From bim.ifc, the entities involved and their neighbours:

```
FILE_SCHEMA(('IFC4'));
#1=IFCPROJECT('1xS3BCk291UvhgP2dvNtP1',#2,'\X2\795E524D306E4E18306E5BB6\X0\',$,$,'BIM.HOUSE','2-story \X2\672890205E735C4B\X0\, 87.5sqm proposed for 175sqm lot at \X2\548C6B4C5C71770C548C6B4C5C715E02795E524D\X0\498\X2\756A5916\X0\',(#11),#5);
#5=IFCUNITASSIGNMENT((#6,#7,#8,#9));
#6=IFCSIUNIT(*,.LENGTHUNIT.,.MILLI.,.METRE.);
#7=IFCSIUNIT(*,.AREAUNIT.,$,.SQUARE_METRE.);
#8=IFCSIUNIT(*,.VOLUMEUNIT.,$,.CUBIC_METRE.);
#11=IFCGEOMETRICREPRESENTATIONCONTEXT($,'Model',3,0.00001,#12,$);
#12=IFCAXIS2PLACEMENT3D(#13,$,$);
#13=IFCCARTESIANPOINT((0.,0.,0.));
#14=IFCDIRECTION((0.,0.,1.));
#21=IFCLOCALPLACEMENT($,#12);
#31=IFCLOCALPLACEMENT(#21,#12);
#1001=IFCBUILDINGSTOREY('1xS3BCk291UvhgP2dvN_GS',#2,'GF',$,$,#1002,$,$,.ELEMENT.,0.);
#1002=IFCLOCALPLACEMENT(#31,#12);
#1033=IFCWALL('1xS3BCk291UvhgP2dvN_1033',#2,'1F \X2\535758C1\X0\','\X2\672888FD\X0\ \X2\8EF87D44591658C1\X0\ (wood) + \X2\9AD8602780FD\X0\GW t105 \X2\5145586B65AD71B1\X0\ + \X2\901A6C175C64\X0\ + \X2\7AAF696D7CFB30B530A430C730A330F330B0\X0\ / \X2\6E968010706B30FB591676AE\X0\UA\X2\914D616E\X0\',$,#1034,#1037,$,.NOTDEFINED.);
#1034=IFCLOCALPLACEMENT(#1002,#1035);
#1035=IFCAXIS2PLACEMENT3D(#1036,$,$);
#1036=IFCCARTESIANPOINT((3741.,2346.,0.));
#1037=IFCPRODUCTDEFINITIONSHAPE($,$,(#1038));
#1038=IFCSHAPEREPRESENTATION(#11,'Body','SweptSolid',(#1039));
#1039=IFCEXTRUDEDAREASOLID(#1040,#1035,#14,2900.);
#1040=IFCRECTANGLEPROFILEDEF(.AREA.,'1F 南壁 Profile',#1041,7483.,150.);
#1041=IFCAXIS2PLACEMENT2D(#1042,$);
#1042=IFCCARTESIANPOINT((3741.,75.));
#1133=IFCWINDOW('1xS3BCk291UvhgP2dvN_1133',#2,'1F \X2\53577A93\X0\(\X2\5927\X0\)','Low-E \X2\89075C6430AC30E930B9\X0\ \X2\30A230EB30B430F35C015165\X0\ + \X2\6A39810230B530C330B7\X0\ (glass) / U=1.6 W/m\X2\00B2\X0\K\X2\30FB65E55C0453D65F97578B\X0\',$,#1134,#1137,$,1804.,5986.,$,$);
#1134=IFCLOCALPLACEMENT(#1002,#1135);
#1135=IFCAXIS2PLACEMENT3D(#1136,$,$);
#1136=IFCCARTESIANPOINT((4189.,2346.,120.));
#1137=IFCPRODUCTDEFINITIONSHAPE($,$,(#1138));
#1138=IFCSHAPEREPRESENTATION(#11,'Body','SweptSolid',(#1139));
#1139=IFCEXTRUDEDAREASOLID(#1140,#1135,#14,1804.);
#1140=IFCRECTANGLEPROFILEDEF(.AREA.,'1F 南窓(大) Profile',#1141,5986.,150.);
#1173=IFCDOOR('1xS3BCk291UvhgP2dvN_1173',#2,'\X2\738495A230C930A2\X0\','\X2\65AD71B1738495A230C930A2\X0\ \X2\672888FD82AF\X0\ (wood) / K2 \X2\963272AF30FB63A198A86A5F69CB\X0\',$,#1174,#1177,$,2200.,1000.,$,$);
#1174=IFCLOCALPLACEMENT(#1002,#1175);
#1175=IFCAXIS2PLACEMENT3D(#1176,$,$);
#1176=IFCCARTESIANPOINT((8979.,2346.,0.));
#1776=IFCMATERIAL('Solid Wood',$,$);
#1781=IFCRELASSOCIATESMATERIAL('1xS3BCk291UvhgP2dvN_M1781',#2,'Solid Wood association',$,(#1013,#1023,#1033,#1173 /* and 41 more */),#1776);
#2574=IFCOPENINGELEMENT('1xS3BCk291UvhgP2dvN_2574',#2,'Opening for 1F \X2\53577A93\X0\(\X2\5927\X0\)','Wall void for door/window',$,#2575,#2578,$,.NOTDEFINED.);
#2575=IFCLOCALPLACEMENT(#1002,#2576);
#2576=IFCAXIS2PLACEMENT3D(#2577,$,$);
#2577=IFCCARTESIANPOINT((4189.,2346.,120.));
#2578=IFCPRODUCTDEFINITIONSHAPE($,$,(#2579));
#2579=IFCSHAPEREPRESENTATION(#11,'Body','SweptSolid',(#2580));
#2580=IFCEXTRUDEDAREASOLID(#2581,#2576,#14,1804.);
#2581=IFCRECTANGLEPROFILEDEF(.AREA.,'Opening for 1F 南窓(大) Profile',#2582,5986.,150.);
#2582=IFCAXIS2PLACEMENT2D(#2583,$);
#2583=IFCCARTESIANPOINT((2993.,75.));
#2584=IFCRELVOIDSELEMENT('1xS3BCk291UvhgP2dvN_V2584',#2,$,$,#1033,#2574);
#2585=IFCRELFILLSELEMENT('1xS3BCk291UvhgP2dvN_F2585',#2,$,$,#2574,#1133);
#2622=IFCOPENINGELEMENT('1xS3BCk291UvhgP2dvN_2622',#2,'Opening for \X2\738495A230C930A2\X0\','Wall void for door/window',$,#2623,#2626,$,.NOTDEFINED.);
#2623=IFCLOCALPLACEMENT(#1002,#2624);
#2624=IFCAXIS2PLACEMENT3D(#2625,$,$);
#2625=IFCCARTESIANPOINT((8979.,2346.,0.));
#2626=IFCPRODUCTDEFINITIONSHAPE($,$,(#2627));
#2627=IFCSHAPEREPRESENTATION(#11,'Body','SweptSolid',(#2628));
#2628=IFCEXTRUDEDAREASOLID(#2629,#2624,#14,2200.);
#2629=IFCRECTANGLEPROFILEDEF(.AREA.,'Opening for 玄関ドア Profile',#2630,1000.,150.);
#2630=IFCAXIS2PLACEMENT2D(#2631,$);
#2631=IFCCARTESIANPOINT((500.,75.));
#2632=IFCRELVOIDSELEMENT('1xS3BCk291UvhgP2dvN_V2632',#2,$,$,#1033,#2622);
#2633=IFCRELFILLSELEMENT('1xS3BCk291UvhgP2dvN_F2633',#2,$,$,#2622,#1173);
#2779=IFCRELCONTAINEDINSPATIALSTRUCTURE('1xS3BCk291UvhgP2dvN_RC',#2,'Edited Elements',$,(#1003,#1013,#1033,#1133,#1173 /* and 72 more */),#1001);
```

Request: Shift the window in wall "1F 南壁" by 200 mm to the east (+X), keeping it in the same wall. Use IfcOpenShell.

```python
import ifcopenshell
import ifcopenshell.api.geometry
import ifcopenshell.util.placement
import ifcopenshell.util.unit

model = ifcopenshell.open("bim.ifc")
unit_scale = ifcopenshell.util.unit.calculate_unit_scale(model)

window = model.by_guid("1xS3BCk291UvhgP2dvN_1133")
opening = window.FillsVoids[0].RelatingOpeningElement
wall = opening.VoidsElements[0].RelatingBuildingElement

wall_matrix = ifcopenshell.util.placement.get_local_placement(wall.ObjectPlacement)
shift = wall_matrix[:3, 0] * 0.2 / unit_scale
before = ifcopenshell.util.placement.get_local_placement(window.ObjectPlacement)[:3, 3].copy()

# The window is not placed relative to its opening, so move both.
for product in (opening, window):
    matrix = ifcopenshell.util.placement.get_local_placement(product.ObjectPlacement)
    matrix[:3, 3] += shift
    ifcopenshell.api.geometry.edit_object_placement(model, product=product, matrix=matrix, is_si=False)

after = ifcopenshell.util.placement.get_local_placement(window.ObjectPlacement)[:3, 3]
print("window moved by", (after - before).round(3) + 0.0)

model.write("bim-out.ifc")
```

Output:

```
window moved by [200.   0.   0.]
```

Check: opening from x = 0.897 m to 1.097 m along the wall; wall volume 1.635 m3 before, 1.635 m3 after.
